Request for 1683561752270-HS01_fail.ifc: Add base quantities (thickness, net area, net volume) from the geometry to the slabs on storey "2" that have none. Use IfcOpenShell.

First a look at what the model holds.

```python
import ifcopenshell
import ifcopenshell.util.element
import ifcopenshell.util.unit

model = ifcopenshell.open("1683561752270-HS01_fail.ifc")
print(model.schema)
for unit_type in ("LENGTHUNIT", "AREAUNIT", "VOLUMEUNIT"):
    print(unit_type, ifcopenshell.util.unit.calculate_unit_scale(model, unit_type))
storey = next(s for s in model.by_type("IfcBuildingStorey") if s.Name == "2")
slabs = [e for e in ifcopenshell.util.element.get_decomposition(storey) if e.is_a("IfcSlab")]
for e in sorted(slabs, key=lambda e: e.id()):
    print(e.id(), e.is_a(), e.Name, list(ifcopenshell.util.element.get_psets(e, qtos_only=True)), sep=" | ")
```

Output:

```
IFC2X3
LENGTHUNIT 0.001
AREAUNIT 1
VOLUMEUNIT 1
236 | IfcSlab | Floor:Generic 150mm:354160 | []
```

```python
import ifcopenshell
import ifcopenshell.api.pset
import ifcopenshell.geom
import ifcopenshell.util.element
import ifcopenshell.util.shape
import ifcopenshell.util.unit

model = ifcopenshell.open("1683561752270-HS01_fail.ifc")
unit_scale = ifcopenshell.util.unit.calculate_unit_scale(model)
area_scale = ifcopenshell.util.unit.calculate_unit_scale(model, "AREAUNIT")
volume_scale = ifcopenshell.util.unit.calculate_unit_scale(model, "VOLUMEUNIT")
settings = ifcopenshell.geom.settings()

storey = next(s for s in model.by_type("IfcBuildingStorey") if s.Name == "2")
slabs = [e for e in ifcopenshell.util.element.get_decomposition(storey) if e.is_a("IfcSlab")]

for e in sorted(slabs, key=lambda e: e.id()):
    if ifcopenshell.util.element.get_psets(e, qtos_only=True, should_inherit=False):
        continue
    # Geometry comes back in metres, in the element's own axes.
    shape = ifcopenshell.geom.create_shape(settings, e)
    values = {
        "Width": ifcopenshell.util.shape.get_z(shape.geometry) / unit_scale,
        "NetArea": ifcopenshell.util.shape.get_footprint_area(shape.geometry) / area_scale,
        "NetVolume": ifcopenshell.util.shape.get_volume(shape.geometry) / volume_scale,
    }
    qto = ifcopenshell.api.pset.add_qto(model, product=e, name="BaseQuantities")
    ifcopenshell.api.pset.edit_qto(model, qto=qto, properties=values)
    print(e.id(), {k: round(v, 3) for k, v in values.items()})

model.write("1683561752270-HS01_fail-out.ifc")
```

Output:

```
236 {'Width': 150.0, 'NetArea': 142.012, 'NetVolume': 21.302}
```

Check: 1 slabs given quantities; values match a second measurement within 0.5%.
